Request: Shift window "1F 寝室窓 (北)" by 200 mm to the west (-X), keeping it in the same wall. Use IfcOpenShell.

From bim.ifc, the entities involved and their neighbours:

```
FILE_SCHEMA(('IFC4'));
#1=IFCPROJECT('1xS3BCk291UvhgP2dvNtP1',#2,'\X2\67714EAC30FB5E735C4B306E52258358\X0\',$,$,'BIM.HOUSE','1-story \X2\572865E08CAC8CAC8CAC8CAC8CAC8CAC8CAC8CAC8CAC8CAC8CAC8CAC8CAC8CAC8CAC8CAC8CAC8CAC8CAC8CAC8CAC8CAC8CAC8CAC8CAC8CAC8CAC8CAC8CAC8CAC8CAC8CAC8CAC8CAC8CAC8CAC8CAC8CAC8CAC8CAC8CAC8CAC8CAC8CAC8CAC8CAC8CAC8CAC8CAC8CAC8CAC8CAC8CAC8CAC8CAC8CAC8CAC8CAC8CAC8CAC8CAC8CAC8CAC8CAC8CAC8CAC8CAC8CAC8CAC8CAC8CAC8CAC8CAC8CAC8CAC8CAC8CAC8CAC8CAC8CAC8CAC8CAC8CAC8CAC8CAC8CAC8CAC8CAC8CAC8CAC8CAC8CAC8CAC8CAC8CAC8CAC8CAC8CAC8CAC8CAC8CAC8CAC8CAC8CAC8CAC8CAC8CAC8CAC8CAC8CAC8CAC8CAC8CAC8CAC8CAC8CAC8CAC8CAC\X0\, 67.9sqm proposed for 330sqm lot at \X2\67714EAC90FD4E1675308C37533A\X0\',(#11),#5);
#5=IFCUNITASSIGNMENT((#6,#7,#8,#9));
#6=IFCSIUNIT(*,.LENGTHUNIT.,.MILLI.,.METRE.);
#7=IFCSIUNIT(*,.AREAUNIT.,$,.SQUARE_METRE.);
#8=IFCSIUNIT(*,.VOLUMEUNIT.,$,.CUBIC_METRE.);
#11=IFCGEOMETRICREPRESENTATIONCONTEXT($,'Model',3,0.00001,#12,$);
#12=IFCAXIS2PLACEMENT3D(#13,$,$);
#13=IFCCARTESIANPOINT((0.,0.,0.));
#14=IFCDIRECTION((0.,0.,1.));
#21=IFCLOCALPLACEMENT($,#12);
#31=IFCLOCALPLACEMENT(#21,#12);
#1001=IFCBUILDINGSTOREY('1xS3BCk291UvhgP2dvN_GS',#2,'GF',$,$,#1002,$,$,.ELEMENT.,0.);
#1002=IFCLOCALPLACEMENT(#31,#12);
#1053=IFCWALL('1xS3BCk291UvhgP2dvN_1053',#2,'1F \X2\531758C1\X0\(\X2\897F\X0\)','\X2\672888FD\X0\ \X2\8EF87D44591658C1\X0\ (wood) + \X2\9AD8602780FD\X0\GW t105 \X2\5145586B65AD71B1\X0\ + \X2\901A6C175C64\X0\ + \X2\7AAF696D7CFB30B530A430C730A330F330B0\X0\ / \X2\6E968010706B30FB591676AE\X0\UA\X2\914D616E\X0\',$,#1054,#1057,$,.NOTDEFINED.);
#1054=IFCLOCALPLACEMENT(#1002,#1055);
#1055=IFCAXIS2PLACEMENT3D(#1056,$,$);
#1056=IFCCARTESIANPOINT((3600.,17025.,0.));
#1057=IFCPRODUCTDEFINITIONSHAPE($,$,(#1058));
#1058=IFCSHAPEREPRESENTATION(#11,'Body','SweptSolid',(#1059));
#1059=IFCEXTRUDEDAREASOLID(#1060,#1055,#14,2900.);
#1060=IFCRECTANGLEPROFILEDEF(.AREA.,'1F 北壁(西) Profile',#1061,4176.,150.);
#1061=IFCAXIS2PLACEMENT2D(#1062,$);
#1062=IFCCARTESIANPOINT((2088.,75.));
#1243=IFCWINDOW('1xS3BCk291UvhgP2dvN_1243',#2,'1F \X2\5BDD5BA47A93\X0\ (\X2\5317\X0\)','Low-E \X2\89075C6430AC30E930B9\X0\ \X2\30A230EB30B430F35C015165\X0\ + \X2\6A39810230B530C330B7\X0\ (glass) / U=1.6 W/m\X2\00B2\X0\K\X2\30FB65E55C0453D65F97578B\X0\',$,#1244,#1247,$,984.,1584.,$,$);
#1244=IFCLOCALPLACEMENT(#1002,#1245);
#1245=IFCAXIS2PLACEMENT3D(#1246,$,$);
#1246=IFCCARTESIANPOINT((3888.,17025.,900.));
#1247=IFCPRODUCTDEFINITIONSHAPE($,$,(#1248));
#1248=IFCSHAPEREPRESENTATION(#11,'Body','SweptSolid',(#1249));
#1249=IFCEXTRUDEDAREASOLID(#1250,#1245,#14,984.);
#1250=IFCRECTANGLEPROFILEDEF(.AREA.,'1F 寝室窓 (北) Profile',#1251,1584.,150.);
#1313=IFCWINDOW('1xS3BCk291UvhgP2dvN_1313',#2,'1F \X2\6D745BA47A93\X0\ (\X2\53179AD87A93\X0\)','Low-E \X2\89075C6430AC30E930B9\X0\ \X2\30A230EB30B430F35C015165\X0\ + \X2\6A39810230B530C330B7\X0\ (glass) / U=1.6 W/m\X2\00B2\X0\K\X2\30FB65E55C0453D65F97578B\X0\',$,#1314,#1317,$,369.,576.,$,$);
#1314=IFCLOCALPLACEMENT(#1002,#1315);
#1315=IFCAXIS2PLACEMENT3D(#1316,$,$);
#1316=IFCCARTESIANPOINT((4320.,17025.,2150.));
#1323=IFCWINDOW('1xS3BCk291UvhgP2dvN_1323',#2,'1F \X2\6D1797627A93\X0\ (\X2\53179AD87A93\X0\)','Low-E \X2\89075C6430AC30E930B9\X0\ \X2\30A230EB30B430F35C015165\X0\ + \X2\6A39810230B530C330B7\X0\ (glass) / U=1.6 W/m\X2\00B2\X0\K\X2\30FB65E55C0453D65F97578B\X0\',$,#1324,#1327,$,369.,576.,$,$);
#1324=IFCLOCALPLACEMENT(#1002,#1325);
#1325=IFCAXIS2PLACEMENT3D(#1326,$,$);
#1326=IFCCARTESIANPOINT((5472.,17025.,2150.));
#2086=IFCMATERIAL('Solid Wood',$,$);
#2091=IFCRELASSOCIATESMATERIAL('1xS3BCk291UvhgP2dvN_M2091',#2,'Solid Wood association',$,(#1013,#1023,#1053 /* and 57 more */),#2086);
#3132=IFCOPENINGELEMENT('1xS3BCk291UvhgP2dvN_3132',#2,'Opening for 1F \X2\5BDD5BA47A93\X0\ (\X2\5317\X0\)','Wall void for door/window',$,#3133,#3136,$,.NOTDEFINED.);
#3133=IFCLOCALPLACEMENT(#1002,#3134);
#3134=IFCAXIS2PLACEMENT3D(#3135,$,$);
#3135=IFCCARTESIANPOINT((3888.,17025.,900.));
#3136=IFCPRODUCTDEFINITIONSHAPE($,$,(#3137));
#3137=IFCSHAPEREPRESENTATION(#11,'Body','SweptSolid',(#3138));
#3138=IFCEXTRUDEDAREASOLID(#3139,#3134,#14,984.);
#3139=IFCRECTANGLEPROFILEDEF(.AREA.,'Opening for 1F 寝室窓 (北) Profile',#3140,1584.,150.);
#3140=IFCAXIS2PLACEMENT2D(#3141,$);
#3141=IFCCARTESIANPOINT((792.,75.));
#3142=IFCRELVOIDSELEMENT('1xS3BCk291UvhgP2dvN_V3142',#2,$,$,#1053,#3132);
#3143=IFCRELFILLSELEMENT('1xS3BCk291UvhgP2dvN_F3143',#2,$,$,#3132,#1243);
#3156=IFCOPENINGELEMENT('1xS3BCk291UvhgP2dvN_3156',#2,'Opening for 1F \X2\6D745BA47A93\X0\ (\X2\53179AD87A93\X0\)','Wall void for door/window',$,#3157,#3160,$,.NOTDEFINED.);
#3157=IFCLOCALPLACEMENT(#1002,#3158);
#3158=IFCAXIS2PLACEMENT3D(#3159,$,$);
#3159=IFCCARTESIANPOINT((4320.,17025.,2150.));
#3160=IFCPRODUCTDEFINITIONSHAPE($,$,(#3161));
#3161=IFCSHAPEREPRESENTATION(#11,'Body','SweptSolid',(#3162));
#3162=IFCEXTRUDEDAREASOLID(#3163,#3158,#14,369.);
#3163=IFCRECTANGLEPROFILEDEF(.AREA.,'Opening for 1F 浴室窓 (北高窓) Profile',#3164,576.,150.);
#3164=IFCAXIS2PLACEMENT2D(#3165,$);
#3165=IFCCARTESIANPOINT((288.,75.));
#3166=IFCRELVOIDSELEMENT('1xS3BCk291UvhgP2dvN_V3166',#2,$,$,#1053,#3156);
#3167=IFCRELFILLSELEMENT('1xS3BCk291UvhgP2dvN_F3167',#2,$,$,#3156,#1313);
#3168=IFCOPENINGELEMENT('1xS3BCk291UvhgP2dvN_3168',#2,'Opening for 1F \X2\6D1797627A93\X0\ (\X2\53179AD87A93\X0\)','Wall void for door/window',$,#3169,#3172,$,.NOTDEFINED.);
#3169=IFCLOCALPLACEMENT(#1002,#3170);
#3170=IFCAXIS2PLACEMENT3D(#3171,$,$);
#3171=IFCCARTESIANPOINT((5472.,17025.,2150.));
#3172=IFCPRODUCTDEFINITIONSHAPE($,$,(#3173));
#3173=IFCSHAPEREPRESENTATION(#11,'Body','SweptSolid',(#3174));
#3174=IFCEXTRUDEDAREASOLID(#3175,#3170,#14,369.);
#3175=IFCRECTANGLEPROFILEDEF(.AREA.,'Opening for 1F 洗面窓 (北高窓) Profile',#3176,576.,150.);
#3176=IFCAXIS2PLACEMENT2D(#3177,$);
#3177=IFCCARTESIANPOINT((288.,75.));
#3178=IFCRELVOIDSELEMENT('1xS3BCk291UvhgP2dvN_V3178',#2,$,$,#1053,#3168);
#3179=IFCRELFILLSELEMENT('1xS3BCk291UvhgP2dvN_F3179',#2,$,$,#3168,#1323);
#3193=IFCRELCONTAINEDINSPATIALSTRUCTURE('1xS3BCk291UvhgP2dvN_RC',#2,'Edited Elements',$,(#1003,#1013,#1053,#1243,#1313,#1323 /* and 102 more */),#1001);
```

```python
import ifcopenshell
import ifcopenshell.api.geometry
import ifcopenshell.util.placement
import ifcopenshell.util.unit

model = ifcopenshell.open("bim.ifc")
unit_scale = ifcopenshell.util.unit.calculate_unit_scale(model)

window = model.by_id(1243)
opening = window.FillsVoids[0].RelatingOpeningElement
wall = opening.VoidsElements[0].RelatingBuildingElement

wall_matrix = ifcopenshell.util.placement.get_local_placement(wall.ObjectPlacement)
shift = wall_matrix[:3, 0] * -0.2 / unit_scale
before = ifcopenshell.util.placement.get_local_placement(window.ObjectPlacement)[:3, 3].copy()

# The window is not placed relative to its opening, so move both.
for product in (opening, window):
    matrix = ifcopenshell.util.placement.get_local_placement(product.ObjectPlacement)
    matrix[:3, 3] += shift
    ifcopenshell.api.geometry.edit_object_placement(model, product=product, matrix=matrix, is_si=False)

after = ifcopenshell.util.placement.get_local_placement(window.ObjectPlacement)[:3, 3]
print("window moved by", (after - before).round(3) + 0.0)

model.write("bim_edited.ifc")
```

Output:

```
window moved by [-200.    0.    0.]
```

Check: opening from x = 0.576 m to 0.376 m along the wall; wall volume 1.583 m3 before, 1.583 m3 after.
